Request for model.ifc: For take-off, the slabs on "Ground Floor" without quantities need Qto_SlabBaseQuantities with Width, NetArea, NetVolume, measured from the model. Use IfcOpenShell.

First a look at what the model holds.

```python
import ifcopenshell
import ifcopenshell.util.element
import ifcopenshell.util.unit

model = ifcopenshell.open("model.ifc")
print(model.schema)
for unit_type in ("LENGTHUNIT", "AREAUNIT", "VOLUMEUNIT"):
    print(unit_type, ifcopenshell.util.unit.calculate_unit_scale(model, unit_type))
storey = next(s for s in model.by_type("IfcBuildingStorey") if s.Name == "Ground Floor")
slabs = [e for e in ifcopenshell.util.element.get_decomposition(storey) if e.is_a("IfcSlab")]
for e in sorted(slabs, key=lambda e: e.id()):
    print(e.id(), e.is_a(), e.Name, list(ifcopenshell.util.element.get_psets(e, qtos_only=True)), sep=" | ")
```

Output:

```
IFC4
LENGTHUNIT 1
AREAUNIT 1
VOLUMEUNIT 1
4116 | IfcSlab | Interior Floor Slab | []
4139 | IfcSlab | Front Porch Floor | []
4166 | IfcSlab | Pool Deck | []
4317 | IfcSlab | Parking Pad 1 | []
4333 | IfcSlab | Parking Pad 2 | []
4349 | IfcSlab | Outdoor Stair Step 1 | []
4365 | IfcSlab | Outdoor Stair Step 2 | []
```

```python
import ifcopenshell
import ifcopenshell.api.pset
import ifcopenshell.geom
import ifcopenshell.util.element
import ifcopenshell.util.shape
import ifcopenshell.util.unit

model = ifcopenshell.open("model.ifc")
unit_scale = ifcopenshell.util.unit.calculate_unit_scale(model)
area_scale = ifcopenshell.util.unit.calculate_unit_scale(model, "AREAUNIT")
volume_scale = ifcopenshell.util.unit.calculate_unit_scale(model, "VOLUMEUNIT")
settings = ifcopenshell.geom.settings()

storey = next(s for s in model.by_type("IfcBuildingStorey") if s.Name == "Ground Floor")
slabs = [e for e in ifcopenshell.util.element.get_decomposition(storey) if e.is_a("IfcSlab")]

for e in sorted(slabs, key=lambda e: e.id()):
    if ifcopenshell.util.element.get_psets(e, qtos_only=True, should_inherit=False):
        continue
    # Geometry comes back in metres, in the element's own axes.
    shape = ifcopenshell.geom.create_shape(settings, e)
    values = {
        "Width": ifcopenshell.util.shape.get_z(shape.geometry) / unit_scale,
        "NetArea": ifcopenshell.util.shape.get_footprint_area(shape.geometry) / area_scale,
        "NetVolume": ifcopenshell.util.shape.get_volume(shape.geometry) / volume_scale,
    }
    qto = ifcopenshell.api.pset.add_qto(model, product=e, name="Qto_SlabBaseQuantities")
    ifcopenshell.api.pset.edit_qto(model, qto=qto, properties=values)
    print(e.id(), {k: round(v, 3) for k, v in values.items()})

model.write("model_updated.ifc")
```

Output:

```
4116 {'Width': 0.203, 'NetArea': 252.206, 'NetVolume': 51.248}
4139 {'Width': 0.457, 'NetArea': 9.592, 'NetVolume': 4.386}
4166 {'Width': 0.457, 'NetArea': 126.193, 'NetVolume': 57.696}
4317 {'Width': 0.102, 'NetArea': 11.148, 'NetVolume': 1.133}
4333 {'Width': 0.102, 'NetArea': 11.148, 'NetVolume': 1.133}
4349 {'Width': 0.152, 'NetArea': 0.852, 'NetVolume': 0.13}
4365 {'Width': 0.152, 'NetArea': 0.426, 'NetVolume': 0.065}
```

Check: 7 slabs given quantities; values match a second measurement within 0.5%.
